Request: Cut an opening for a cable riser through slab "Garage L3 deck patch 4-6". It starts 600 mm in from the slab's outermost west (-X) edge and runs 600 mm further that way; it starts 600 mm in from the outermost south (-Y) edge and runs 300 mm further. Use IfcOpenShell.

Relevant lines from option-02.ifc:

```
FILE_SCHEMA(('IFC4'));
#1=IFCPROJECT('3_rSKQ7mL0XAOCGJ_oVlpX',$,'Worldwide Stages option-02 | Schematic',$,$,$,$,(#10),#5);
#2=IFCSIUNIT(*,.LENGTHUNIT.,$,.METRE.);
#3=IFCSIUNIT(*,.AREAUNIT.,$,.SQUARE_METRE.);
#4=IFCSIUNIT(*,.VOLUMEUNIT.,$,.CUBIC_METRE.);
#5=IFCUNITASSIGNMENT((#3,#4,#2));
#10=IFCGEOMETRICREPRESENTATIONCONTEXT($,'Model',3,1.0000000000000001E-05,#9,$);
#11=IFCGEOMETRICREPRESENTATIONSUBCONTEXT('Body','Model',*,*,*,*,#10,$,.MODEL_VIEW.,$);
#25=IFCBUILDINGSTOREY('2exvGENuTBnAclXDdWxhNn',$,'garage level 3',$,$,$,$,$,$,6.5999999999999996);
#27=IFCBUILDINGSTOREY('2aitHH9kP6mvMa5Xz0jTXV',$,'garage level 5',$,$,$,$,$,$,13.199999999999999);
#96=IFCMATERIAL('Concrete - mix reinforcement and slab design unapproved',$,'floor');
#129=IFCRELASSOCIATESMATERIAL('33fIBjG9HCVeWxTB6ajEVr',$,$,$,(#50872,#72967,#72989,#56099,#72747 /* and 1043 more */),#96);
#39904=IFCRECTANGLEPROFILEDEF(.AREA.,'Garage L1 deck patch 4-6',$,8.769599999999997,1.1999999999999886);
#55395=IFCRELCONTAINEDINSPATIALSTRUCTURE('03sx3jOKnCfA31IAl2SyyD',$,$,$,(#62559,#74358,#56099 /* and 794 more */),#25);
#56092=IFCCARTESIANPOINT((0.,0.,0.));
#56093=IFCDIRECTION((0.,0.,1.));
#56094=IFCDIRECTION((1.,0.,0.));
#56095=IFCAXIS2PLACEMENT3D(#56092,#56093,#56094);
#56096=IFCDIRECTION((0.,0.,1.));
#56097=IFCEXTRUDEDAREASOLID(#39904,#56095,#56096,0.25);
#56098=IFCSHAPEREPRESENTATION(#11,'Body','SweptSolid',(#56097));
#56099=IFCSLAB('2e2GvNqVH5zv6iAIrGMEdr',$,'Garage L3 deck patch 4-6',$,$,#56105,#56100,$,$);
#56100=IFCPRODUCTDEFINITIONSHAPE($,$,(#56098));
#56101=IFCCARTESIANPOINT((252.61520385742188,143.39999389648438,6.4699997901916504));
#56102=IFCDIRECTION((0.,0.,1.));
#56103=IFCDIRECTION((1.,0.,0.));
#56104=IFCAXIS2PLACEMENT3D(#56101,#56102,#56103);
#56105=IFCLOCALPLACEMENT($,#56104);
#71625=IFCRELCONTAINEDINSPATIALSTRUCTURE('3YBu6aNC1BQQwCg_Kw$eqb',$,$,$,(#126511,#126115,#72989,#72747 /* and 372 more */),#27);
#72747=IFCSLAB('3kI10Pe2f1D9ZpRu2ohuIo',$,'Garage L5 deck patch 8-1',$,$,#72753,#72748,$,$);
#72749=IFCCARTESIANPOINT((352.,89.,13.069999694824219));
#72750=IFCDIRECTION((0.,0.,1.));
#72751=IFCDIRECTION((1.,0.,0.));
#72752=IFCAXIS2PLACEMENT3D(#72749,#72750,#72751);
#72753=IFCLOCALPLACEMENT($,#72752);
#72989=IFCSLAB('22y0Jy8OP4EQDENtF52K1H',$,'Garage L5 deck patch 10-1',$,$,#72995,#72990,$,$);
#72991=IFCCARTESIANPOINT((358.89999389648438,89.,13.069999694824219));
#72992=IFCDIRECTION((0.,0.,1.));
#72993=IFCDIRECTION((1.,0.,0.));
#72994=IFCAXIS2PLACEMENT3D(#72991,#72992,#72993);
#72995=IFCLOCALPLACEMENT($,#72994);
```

```python
import numpy as np
import ifcopenshell
import ifcopenshell.api.feature
import ifcopenshell.api.geometry
import ifcopenshell.api.root
import ifcopenshell.geom
import ifcopenshell.util.placement
import ifcopenshell.util.representation
import ifcopenshell.util.shape
import ifcopenshell.util.unit

model = ifcopenshell.open("option-02.ifc")
unit_scale = ifcopenshell.util.unit.calculate_unit_scale(model)
settings = ifcopenshell.geom.settings()


def volume(element):
    """Net volume in cubic metres, openings subtracted."""
    shape = ifcopenshell.geom.create_shape(settings, element)
    return ifcopenshell.util.shape.get_volume(shape.geometry)


slab = model.by_id(56099)
before = volume(slab)

# Extent in the slab's own axes, in metres. The edges named are its -X and -Y sides.
slab_shape = ifcopenshell.geom.create_shape(settings, slab)
vertices = ifcopenshell.util.shape.get_vertices(slab_shape.geometry)
x_min, y_min, bottom = vertices.min(axis=0)
top = vertices[:, 2].max()

opening = ifcopenshell.api.root.create_entity(model, ifc_class="IfcOpeningElement", name="Cable riser opening", predefined_type="OPENING")
context = ifcopenshell.util.representation.get_context(model, "Model", "Body", "MODEL_VIEW")
width, depth = 0.6, 0.3
outline = [(0.0, 0.0), (width, 0.0), (width, depth), (0.0, depth), (0.0, 0.0)]
# Overshoot both faces by 50 mm so the cut is clean.
shape = ifcopenshell.api.geometry.add_slab_representation(
    model, context=context, depth=top - bottom + 0.1, polyline=outline
)
ifcopenshell.api.geometry.assign_representation(model, product=opening, representation=shape)

matrix = ifcopenshell.util.placement.get_local_placement(slab.ObjectPlacement)
matrix[:, 3] = matrix @ np.append(np.array([x_min + 0.6, y_min + 0.6, bottom - 0.05]) / unit_scale, 1.0)
ifcopenshell.api.geometry.edit_object_placement(model, product=opening, matrix=matrix, is_si=False)
ifcopenshell.api.feature.add_feature(model, feature=opening, element=slab)

after = volume(slab)

print(f"slab volume {before:.3f} -> {after:.3f} m3")

model.write("option-02_updated.ifc")
```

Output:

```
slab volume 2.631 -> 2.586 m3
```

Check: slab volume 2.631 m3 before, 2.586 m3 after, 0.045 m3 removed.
